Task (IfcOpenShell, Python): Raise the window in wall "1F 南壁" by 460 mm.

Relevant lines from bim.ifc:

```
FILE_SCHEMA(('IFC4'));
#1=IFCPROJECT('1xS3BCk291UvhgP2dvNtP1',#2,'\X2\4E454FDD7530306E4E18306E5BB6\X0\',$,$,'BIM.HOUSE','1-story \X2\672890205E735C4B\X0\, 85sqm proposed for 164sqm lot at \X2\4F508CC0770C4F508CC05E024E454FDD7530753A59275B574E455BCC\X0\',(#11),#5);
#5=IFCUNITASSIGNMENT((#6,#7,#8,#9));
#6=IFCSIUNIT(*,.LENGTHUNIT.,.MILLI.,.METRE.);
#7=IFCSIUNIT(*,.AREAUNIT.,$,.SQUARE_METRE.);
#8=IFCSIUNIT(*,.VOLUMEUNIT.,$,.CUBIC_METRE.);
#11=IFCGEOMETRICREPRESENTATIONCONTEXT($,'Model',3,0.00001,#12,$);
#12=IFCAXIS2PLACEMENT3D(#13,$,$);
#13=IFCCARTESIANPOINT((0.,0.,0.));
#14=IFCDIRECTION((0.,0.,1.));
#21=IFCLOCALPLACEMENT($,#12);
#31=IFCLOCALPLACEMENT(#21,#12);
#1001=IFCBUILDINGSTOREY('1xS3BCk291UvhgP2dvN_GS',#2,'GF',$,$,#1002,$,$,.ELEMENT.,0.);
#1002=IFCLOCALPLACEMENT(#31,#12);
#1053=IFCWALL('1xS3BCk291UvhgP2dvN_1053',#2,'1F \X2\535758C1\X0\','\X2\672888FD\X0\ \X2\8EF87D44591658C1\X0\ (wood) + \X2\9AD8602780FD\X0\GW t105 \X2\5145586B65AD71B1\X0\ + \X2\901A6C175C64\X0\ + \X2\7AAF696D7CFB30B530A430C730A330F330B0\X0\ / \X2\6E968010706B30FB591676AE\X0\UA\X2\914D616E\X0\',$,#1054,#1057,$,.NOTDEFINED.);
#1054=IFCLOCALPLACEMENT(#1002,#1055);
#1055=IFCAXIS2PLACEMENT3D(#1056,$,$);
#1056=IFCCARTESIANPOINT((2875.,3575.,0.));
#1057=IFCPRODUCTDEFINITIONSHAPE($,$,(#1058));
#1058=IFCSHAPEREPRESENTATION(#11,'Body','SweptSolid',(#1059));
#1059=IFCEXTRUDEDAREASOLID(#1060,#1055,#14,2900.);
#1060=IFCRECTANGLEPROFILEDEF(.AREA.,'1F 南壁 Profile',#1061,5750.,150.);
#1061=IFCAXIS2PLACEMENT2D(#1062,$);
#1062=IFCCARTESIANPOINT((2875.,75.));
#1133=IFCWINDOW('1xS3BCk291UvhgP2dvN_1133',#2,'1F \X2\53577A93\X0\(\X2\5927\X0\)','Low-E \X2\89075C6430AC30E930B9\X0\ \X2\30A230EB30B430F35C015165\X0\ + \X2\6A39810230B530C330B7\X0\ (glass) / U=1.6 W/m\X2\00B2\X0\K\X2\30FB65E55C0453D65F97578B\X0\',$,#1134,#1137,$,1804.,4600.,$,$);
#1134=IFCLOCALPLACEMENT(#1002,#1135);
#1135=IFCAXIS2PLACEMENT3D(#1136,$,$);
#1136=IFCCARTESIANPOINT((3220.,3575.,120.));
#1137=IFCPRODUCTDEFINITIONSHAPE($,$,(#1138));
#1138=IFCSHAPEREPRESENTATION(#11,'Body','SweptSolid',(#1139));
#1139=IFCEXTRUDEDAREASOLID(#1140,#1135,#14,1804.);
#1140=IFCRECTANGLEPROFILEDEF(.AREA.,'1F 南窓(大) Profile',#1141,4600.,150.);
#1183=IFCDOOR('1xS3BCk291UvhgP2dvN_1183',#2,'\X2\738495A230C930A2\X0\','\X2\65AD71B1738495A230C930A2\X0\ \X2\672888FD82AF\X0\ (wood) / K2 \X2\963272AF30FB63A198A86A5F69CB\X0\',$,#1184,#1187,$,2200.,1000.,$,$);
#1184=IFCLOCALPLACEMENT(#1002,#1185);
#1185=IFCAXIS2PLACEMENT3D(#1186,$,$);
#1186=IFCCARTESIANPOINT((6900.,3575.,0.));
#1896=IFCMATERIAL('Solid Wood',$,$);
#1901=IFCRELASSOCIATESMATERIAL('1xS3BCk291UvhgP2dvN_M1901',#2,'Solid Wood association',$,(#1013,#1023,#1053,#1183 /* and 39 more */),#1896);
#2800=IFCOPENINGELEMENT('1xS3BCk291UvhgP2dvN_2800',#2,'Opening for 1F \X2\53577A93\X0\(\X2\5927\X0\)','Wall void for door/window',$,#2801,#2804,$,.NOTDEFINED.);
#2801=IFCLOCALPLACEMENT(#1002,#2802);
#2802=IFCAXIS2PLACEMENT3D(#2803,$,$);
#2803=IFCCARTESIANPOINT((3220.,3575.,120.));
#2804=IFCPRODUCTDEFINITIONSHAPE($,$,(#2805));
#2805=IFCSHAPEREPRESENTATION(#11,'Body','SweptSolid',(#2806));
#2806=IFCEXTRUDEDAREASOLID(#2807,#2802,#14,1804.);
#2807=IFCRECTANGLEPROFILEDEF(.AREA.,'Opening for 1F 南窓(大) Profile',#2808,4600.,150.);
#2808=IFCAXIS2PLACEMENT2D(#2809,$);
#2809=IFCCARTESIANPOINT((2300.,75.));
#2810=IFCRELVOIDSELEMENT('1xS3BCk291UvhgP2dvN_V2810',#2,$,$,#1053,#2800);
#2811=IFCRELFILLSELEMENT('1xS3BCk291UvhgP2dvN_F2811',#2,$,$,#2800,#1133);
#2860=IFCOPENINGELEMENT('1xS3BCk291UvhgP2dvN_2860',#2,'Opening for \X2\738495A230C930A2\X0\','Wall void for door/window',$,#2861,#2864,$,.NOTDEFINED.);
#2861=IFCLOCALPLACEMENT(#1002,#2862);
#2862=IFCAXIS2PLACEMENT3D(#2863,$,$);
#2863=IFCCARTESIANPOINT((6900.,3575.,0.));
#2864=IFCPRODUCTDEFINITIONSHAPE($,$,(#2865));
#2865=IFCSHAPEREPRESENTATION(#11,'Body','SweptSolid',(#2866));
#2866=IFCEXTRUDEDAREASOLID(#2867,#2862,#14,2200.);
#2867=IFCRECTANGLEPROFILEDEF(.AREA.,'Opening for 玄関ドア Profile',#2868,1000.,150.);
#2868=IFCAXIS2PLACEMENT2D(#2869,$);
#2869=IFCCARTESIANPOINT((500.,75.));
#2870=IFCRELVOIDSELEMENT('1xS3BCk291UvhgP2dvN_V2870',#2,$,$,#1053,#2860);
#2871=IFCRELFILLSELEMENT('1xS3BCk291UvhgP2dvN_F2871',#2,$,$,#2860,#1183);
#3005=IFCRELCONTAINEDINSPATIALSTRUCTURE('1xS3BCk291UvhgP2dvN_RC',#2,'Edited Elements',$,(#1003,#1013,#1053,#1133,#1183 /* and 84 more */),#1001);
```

```python
import numpy as np
import ifcopenshell
import ifcopenshell.api.geometry
import ifcopenshell.util.placement
import ifcopenshell.util.unit

model = ifcopenshell.open("bim.ifc")
unit_scale = ifcopenshell.util.unit.calculate_unit_scale(model)

window = model.by_id(1133)
opening = window.FillsVoids[0].RelatingOpeningElement
dz = 0.46 / unit_scale

shift = np.array([0.0, 0.0, dz])
# The window is not placed relative to its opening, so move both.
for product in (opening, window):
    matrix = ifcopenshell.util.placement.get_local_placement(product.ObjectPlacement)
    matrix[:3, 3] += shift
    ifcopenshell.api.geometry.edit_object_placement(model, product=product, matrix=matrix, is_si=False)

print(f"moved by {dz * unit_scale:+.3f} m")

model.write("bim-out.ifc")
```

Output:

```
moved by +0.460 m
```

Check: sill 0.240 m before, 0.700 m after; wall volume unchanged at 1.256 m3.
